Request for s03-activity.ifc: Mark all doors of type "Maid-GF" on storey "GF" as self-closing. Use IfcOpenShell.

First a look at what the model holds.

```python
import ifcopenshell
import ifcopenshell.util.element

model = ifcopenshell.open("s03-activity.ifc")
print(model.schema)
storey = next(s for s in model.by_type("IfcBuildingStorey") if s.Name == "GF")
doors = [e for e in ifcopenshell.util.element.get_decomposition(storey) if e.is_a("IfcDoor")]
seen = {}
for e in doors:
    element_type = ifcopenshell.util.element.get_type(e)
    key = (element_type.Name if element_type != e and element_type else None, ifcopenshell.util.element.get_pset(e, "Pset_DoorCommon", "SelfClosing"))
    seen[key] = seen.get(key, 0) + 1
for (name, value), count in sorted(seen.items(), key=str):
    print(count, "x", name, "|", value)
```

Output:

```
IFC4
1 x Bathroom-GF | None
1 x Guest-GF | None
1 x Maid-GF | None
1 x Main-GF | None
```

```python
import ifcopenshell
import ifcopenshell.api.pset
import ifcopenshell.util.element

model = ifcopenshell.open("s03-activity.ifc")

storey = next(s for s in model.by_type("IfcBuildingStorey") if s.Name == "GF")
doors = [e for e in ifcopenshell.util.element.get_decomposition(storey) if e.is_a("IfcDoor")]

count = 0
for e in doors:
    element_type = ifcopenshell.util.element.get_type(e)
    if element_type in (None, e) or element_type.Name != "Maid-GF":
        continue
    # add_pset returns the element's existing set when there is one.
    pset = ifcopenshell.api.pset.add_pset(model, product=e, name="Pset_DoorCommon")
    ifcopenshell.api.pset.edit_pset(model, pset=pset, properties={"SelfClosing": True})
    count += 1

print(count, "doors updated")

model.write("s03-activity-out.ifc")
```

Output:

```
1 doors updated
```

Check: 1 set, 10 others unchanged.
